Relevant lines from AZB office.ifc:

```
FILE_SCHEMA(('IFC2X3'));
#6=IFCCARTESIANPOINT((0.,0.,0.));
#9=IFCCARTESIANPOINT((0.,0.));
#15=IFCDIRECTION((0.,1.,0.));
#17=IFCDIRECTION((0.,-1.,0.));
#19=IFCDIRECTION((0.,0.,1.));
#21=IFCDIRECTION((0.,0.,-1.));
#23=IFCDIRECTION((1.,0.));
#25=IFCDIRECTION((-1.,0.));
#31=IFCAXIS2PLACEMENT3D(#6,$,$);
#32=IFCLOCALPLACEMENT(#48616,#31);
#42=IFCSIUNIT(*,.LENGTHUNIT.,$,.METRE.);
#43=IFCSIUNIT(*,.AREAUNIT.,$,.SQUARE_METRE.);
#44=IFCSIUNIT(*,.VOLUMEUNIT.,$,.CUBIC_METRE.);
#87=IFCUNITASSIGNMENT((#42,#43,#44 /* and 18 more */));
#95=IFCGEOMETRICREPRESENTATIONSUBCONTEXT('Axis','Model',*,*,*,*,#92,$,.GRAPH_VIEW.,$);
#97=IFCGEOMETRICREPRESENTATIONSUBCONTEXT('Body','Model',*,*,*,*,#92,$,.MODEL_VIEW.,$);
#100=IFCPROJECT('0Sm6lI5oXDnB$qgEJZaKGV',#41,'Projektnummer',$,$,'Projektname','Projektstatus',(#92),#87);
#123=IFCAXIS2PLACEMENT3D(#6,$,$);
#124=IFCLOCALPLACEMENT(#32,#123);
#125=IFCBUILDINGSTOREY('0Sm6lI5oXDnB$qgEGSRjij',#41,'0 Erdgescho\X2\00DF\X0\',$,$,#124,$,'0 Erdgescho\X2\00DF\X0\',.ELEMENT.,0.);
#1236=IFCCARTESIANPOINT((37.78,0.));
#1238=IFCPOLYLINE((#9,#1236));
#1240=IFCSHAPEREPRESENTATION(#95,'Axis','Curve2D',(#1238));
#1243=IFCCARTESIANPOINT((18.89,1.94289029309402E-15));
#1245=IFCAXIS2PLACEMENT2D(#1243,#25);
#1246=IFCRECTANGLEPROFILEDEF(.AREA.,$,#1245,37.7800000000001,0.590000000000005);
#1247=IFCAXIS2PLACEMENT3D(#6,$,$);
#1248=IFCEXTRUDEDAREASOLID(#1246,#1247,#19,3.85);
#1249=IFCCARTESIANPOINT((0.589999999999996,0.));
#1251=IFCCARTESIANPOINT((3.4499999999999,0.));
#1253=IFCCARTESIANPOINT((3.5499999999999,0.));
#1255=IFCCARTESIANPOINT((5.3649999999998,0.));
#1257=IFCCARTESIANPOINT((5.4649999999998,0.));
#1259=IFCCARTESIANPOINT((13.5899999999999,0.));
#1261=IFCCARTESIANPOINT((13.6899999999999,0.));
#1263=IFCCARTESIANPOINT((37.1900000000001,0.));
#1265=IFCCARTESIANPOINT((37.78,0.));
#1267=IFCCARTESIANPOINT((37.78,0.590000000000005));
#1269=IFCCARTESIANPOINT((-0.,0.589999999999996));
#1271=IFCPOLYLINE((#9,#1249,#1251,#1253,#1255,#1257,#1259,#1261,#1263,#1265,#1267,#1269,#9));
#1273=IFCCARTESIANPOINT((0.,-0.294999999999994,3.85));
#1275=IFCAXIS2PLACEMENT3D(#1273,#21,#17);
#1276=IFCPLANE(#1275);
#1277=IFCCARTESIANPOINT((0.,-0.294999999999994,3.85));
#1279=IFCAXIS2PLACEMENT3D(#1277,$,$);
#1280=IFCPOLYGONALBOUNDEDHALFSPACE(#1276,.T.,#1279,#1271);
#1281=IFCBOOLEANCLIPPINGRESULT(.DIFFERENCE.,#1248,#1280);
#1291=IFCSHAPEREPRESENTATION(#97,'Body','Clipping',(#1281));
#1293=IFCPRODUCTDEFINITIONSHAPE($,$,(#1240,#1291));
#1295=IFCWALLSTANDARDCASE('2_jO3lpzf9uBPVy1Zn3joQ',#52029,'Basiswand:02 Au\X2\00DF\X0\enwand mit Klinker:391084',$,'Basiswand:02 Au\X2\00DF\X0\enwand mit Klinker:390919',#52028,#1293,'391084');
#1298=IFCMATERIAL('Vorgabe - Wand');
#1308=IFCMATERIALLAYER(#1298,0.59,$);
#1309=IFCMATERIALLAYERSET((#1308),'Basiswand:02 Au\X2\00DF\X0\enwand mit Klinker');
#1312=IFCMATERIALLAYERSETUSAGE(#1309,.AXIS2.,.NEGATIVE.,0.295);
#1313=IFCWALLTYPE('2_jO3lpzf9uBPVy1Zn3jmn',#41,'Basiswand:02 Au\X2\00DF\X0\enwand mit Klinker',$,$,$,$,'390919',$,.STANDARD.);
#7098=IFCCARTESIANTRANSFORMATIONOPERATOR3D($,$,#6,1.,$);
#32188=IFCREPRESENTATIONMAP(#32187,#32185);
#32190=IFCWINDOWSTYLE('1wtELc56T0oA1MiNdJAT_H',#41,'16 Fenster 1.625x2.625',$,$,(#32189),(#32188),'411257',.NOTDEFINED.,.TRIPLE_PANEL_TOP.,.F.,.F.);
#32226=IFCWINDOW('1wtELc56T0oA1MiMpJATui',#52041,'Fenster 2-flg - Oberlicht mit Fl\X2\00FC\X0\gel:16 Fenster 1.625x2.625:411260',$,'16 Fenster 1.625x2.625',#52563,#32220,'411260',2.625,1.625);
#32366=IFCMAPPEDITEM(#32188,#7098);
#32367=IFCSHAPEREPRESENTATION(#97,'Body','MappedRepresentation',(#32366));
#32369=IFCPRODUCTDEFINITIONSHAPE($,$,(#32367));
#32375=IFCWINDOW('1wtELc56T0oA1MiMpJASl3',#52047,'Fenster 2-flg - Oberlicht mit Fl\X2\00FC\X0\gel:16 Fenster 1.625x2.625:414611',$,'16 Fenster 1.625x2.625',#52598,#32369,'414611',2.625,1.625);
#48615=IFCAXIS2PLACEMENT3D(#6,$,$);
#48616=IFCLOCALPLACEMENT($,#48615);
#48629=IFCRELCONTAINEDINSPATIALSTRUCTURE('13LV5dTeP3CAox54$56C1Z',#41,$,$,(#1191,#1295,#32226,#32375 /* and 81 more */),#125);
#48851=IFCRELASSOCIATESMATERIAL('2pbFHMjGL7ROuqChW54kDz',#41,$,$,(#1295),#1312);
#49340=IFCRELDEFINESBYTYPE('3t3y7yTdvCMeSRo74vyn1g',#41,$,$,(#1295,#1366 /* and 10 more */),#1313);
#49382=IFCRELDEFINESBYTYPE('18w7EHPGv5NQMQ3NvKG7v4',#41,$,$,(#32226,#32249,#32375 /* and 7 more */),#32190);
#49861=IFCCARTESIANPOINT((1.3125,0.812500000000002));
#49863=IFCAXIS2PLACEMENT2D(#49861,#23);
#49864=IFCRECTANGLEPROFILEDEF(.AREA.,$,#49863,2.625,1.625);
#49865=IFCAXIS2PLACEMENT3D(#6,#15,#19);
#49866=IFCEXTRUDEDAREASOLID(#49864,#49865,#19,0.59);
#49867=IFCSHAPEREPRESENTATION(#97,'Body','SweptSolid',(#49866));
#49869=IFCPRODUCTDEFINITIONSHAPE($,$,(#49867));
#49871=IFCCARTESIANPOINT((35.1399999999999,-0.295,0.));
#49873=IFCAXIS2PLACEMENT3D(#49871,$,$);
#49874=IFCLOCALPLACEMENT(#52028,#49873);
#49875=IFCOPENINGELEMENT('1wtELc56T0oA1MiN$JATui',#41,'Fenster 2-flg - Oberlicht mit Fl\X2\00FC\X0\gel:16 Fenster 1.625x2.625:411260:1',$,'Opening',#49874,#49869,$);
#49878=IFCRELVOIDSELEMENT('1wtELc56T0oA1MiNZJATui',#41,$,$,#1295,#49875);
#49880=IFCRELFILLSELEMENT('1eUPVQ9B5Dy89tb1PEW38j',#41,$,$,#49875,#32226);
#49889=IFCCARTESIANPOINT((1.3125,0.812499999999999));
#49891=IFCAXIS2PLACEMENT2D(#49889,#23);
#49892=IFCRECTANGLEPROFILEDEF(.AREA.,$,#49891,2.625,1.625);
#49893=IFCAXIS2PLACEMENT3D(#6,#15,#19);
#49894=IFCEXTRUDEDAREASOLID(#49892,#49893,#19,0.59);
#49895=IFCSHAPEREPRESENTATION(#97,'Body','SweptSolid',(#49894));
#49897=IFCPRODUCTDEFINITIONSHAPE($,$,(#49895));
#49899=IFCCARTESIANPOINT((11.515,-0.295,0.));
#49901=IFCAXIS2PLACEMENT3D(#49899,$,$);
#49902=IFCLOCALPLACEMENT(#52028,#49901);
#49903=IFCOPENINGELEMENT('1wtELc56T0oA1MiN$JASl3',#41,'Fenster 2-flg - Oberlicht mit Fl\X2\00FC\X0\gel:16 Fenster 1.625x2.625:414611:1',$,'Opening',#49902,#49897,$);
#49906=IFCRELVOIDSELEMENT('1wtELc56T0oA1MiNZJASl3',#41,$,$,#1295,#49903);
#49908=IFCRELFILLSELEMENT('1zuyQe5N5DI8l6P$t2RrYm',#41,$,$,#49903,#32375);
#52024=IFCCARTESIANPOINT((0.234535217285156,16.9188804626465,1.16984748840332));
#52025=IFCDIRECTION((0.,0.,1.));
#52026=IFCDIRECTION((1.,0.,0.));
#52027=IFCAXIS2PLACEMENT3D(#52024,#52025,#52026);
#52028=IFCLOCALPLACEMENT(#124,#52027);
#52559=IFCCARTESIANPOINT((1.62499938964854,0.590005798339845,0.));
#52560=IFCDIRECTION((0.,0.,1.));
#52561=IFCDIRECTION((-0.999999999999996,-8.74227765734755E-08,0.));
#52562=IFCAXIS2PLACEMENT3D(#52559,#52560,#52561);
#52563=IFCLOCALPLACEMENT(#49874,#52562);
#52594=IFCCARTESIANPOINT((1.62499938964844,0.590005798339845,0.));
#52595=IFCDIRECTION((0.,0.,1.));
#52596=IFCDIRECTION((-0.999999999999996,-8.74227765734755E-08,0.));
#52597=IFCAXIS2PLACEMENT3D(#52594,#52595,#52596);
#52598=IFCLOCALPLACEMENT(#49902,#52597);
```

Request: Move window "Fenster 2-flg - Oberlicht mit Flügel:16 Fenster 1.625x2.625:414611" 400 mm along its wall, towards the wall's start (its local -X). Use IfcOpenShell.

```python
import ifcopenshell
import ifcopenshell.api.geometry
import ifcopenshell.util.placement
import ifcopenshell.util.unit

model = ifcopenshell.open("AZB office.ifc")
unit_scale = ifcopenshell.util.unit.calculate_unit_scale(model)

window = model.by_guid("1wtELc56T0oA1MiMpJASl3")
opening = window.FillsVoids[0].RelatingOpeningElement
wall = opening.VoidsElements[0].RelatingBuildingElement

wall_matrix = ifcopenshell.util.placement.get_local_placement(wall.ObjectPlacement)
shift = wall_matrix[:3, 0] * -0.4 / unit_scale
before = ifcopenshell.util.placement.get_local_placement(window.ObjectPlacement)[:3, 3].copy()

# The window is placed relative to its opening, so it follows when the opening moves.
matrix = ifcopenshell.util.placement.get_local_placement(opening.ObjectPlacement)
matrix[:3, 3] += shift
ifcopenshell.api.geometry.edit_object_placement(
    model, product=opening, matrix=matrix, is_si=False, should_transform_children=True
)

after = ifcopenshell.util.placement.get_local_placement(window.ObjectPlacement)[:3, 3]
print("window moved by", (after - before).round(3) + 0.0)

model.write("AZB office_edited.ifc")
```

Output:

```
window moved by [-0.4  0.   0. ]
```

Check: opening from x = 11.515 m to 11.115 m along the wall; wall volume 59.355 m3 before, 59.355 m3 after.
